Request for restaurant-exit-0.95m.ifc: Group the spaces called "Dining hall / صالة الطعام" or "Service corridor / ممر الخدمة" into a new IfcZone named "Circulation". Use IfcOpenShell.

First a look at what the model holds.

```python
import ifcopenshell

model = ifcopenshell.open("restaurant-exit-0.95m.ifc")
print(model.schema)
seen = {}
for space in model.by_type("IfcSpace"):
    seen[space.LongName] = seen.get(space.LongName, 0) + 1
for name, count in sorted(seen.items(), key=str):
    print(count, "x", name)
print("zones:", [z.Name for z in model.by_type("IfcZone")][:20])
```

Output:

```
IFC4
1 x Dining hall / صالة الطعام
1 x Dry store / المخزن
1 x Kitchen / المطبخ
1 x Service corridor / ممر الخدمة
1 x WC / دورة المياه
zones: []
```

```python
import ifcopenshell
import ifcopenshell.api.group
import ifcopenshell.api.root

model = ifcopenshell.open("restaurant-exit-0.95m.ifc")

names = {"Dining hall / صالة الطعام", "Service corridor / ممر الخدمة"}
spaces = [s for s in model.by_type("IfcSpace") if s.LongName in names]

zone = ifcopenshell.api.root.create_entity(model, ifc_class="IfcZone", name="Circulation")
ifcopenshell.api.group.assign_group(model, products=spaces, group=zone)
print(len(spaces), "spaces in", zone.Name)

model.write("restaurant-exit-0.95m_v2.ifc")
```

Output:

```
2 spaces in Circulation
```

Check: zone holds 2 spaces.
